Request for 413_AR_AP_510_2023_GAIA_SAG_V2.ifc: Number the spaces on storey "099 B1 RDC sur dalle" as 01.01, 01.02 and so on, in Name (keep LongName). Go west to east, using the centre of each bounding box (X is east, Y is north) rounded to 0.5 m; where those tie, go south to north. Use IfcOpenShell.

First a look at what the model holds.

```python
import ifcopenshell
import ifcopenshell.util.element
import ifcopenshell.util.placement

model = ifcopenshell.open("413_AR_AP_510_2023_GAIA_SAG_V2.ifc")
print(model.schema)
storey = next(s for s in model.by_type("IfcBuildingStorey") if s.Name == "099 B1 RDC sur dalle")
spaces = [e for e in ifcopenshell.util.element.get_decomposition(storey) if e.is_a("IfcSpace")]
for e in sorted(spaces, key=lambda e: e.id()):
    origin = ifcopenshell.util.placement.get_local_placement(e.ObjectPlacement)[:3, 3]
    print(e.id(), e.Name, e.LongName, origin.round(2) + 0.0, sep=" | ")
```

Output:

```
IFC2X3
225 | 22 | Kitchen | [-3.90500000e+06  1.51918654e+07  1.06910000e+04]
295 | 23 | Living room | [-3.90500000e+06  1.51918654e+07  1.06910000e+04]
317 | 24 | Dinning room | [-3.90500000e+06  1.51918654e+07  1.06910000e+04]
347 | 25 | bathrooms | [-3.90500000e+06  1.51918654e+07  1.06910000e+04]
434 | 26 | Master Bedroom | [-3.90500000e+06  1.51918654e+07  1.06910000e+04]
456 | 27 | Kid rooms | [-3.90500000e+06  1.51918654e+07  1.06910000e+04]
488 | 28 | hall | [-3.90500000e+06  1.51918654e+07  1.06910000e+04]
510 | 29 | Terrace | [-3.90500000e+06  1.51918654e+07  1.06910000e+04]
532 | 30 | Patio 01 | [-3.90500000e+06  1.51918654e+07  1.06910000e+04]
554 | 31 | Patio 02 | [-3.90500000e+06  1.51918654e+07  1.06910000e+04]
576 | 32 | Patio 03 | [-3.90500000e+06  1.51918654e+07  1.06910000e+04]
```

```python
import ifcopenshell
import ifcopenshell.geom
import ifcopenshell.util.element
import ifcopenshell.util.shape

model = ifcopenshell.open("413_AR_AP_510_2023_GAIA_SAG_V2.ifc")
settings = ifcopenshell.geom.settings()
settings.set("use-world-coords", True)


def centre(element):
    shape = ifcopenshell.geom.create_shape(settings, element)
    return ifcopenshell.util.shape.get_bbox_centroid(shape.geometry)


storey = next(s for s in model.by_type("IfcBuildingStorey") if s.Name == "099 B1 RDC sur dalle")
spaces = [e for e in ifcopenshell.util.element.get_decomposition(storey) if e.is_a("IfcSpace")]

# Insertion points can sit at a corner or the storey origin, so sort by the geometry (in metres).
centres = {e: centre(e) for e in spaces}
spaces.sort(key=lambda e: (round(centres[e][0] / 0.5), centres[e][1]))

for i, e in enumerate(spaces, start=1):
    number = f"01.{i:02d}"
    e.Name = number
    print(e.id(), number)

model.write("413_AR_AP_510_2023_GAIA_SAG_V2_edited.ifc")
```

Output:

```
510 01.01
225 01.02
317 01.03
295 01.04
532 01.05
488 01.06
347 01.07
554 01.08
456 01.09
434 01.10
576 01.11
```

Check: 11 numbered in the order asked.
